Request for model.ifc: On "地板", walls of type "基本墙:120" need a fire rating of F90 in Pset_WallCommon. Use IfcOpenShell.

First a look at what the model holds.

```python
import ifcopenshell
import ifcopenshell.util.element

model = ifcopenshell.open("model.ifc")
print(model.schema)
storey = next(s for s in model.by_type("IfcBuildingStorey") if s.Name == "地板")
walls = [e for e in ifcopenshell.util.element.get_decomposition(storey) if e.is_a("IfcWall")]
seen = {}
for e in walls:
    element_type = ifcopenshell.util.element.get_type(e)
    key = (element_type.Name if element_type != e and element_type else None, ifcopenshell.util.element.get_pset(e, "Pset_WallCommon", "FireRating"))
    seen[key] = seen.get(key, 0) + 1
for (name, value), count in sorted(seen.items(), key=str):
    print(count, "x", name, "|", value)
```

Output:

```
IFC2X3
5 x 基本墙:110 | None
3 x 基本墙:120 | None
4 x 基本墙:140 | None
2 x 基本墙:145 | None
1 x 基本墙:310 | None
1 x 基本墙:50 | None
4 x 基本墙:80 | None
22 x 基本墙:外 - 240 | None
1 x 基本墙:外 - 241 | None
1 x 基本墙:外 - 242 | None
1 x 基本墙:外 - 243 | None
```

```python
import ifcopenshell
import ifcopenshell.api.pset
import ifcopenshell.util.element

model = ifcopenshell.open("model.ifc")

storey = next(s for s in model.by_type("IfcBuildingStorey") if s.Name == "地板")
walls = [e for e in ifcopenshell.util.element.get_decomposition(storey) if e.is_a("IfcWall")]

count = 0
for e in walls:
    element_type = ifcopenshell.util.element.get_type(e)
    if element_type in (None, e) or element_type.Name != "基本墙:120":
        continue
    # add_pset returns the element's existing set when there is one.
    pset = ifcopenshell.api.pset.add_pset(model, product=e, name="Pset_WallCommon")
    ifcopenshell.api.pset.edit_pset(model, pset=pset, properties={"FireRating": "F90"})
    count += 1

print(count, "walls updated")

model.write("model_rev.ifc")
```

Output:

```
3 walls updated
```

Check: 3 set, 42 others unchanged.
